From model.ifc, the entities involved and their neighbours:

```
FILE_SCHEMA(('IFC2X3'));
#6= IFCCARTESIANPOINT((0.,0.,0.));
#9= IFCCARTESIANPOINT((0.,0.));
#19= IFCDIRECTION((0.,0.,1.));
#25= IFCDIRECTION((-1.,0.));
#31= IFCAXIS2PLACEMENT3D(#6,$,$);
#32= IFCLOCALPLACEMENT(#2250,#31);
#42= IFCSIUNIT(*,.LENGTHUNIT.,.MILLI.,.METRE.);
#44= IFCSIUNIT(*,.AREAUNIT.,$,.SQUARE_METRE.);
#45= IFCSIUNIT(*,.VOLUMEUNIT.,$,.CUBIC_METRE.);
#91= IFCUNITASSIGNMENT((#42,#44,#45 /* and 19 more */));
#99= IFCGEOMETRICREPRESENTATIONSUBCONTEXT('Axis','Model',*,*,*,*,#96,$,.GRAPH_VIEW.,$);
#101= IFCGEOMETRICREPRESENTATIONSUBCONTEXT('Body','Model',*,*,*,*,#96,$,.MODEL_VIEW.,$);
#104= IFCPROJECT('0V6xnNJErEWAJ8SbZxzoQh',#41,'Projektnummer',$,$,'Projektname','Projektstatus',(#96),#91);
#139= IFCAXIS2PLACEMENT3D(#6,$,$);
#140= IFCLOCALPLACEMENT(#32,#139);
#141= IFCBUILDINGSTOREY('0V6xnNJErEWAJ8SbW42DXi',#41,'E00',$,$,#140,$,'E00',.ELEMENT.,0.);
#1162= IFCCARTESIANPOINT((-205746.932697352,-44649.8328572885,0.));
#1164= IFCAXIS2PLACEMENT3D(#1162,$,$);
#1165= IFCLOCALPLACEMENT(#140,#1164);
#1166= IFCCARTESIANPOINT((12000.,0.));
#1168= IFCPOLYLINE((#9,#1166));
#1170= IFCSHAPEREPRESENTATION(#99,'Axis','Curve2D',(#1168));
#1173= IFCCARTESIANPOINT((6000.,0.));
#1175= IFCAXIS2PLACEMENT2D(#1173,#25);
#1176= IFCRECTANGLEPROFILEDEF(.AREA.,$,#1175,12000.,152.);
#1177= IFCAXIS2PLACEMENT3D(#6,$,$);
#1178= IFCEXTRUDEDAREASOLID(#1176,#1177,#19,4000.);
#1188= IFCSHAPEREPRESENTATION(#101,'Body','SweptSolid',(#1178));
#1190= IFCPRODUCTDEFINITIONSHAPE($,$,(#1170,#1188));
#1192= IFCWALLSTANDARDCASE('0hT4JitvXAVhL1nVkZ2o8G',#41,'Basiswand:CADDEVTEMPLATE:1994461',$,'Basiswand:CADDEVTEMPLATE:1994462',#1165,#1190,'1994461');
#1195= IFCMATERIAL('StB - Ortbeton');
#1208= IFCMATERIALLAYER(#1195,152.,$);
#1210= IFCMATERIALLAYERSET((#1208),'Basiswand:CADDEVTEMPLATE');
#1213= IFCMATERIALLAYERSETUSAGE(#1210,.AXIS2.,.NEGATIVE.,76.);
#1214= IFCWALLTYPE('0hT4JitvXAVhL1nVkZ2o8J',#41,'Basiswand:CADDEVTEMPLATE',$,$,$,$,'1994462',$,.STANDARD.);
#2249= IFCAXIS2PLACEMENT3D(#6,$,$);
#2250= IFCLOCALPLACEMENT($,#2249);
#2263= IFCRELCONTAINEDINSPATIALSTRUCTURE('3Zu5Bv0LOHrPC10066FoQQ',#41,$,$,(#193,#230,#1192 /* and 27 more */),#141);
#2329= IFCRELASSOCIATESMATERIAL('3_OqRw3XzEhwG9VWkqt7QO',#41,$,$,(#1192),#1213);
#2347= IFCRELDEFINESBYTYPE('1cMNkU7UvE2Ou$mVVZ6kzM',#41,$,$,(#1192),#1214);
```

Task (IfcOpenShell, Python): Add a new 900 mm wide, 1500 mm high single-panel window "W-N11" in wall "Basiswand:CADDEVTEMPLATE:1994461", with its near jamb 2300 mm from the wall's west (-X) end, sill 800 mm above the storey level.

```python
import numpy as np
import ifcopenshell
import ifcopenshell.api.feature
import ifcopenshell.api.geometry
import ifcopenshell.api.root
import ifcopenshell.api.spatial
import ifcopenshell.api.type
import ifcopenshell.geom
import ifcopenshell.util.element
import ifcopenshell.util.placement
import ifcopenshell.util.representation
import ifcopenshell.util.shape
import ifcopenshell.util.unit

model = ifcopenshell.open("model.ifc")
unit_scale = ifcopenshell.util.unit.calculate_unit_scale(model)
settings = ifcopenshell.geom.settings()


def volume(element):
    """Net volume in cubic metres, openings subtracted."""
    shape = ifcopenshell.geom.create_shape(settings, element)
    return ifcopenshell.util.shape.get_volume(shape.geometry)


wall = model.by_guid("0hT4JitvXAVhL1nVkZ2o8G")
storey = ifcopenshell.util.element.get_container(wall, ifc_class="IfcBuildingStorey")
context = ifcopenshell.util.representation.get_context(model, "Model", "Body", "MODEL_VIEW")
before = volume(wall)

width, height, from_end, sill = 0.9, 1.5, 2.3, 0.8  # metres

# The wall runs along its own X axis, and the end named is its -X end.
wall_shape = ifcopenshell.geom.create_shape(settings, wall)
x, y, z = ifcopenshell.util.shape.get_vertices(wall_shape.geometry).T
start = x.min() + from_end
face, thickness = float(y.min()), float(y.max() - y.min())
wall_matrix = ifcopenshell.util.placement.get_local_placement(wall.ObjectPlacement)
level = ifcopenshell.util.placement.get_local_placement(storey.ObjectPlacement)[2, 3]


def in_wall(x, y):
    """Placement at x, y metres in the wall's axes, at sill height."""
    matrix = wall_matrix.copy()
    matrix[:, 3] = wall_matrix @ np.array([x / unit_scale, y / unit_scale, 0.0, 1.0])
    matrix[2, 3] = level + sill / unit_scale
    return matrix


# Opening: a box that overshoots both wall faces by 50 mm.
opening = ifcopenshell.api.root.create_entity(model, ifc_class="IfcOpeningElement")
box = ifcopenshell.api.geometry.add_wall_representation(
    model, context=context, length=width, height=height, thickness=thickness + 0.1
)
ifcopenshell.api.geometry.assign_representation(model, product=opening, representation=box)
ifcopenshell.api.geometry.edit_object_placement(model, product=opening, matrix=in_wall(start, face - 0.05), is_si=False)
ifcopenshell.api.feature.add_feature(model, feature=opening, element=wall)

window = ifcopenshell.api.root.create_entity(model, ifc_class="IfcWindow", name="W-N11")
window.OverallWidth, window.OverallHeight = width / unit_scale, height / unit_scale
body = ifcopenshell.api.geometry.add_window_representation(
    model,
    context=context,
    overall_width=window.OverallWidth,
    overall_height=window.OverallHeight,
    partition_type="SINGLE_PANEL",
)
ifcopenshell.api.geometry.assign_representation(model, product=window, representation=body)
ifcopenshell.api.spatial.assign_container(model, products=[window], relating_structure=storey)
fills = ifcopenshell.api.feature.add_filling(model, opening=opening, element=window)
fills.OwnerHistory = window.OwnerHistory  # required in IFC2X3

# IFC2X3 keeps the operation on the window style.
style = ifcopenshell.api.root.create_entity(model, ifc_class="IfcWindowStyle", name="W-N11")
style.OperationType, style.ConstructionType = "SINGLE_PANEL", "NOTDEFINED"
style.ParameterTakesPrecedence = style.Sizeable = False
ifcopenshell.api.type.assign_type(model, related_objects=[window], relating_type=style)

# Centre the window in the wall's thickness.
ifcopenshell.api.geometry.edit_object_placement(model, product=window, matrix=in_wall(start, face), is_si=False)
window_shape = ifcopenshell.geom.create_shape(settings, window)
depth = ifcopenshell.util.shape.get_vertices(window_shape.geometry)[:, 1]
offset = face + thickness / 2 - (depth.min() + depth.max()) / 2
ifcopenshell.api.geometry.edit_object_placement(model, product=window, matrix=in_wall(start, offset), is_si=False)

after = volume(wall)

print(f"wall volume {before:.3f} -> {after:.3f} m3")

model.write("model_v2.ifc")
```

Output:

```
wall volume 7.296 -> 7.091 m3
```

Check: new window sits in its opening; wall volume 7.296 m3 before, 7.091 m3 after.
